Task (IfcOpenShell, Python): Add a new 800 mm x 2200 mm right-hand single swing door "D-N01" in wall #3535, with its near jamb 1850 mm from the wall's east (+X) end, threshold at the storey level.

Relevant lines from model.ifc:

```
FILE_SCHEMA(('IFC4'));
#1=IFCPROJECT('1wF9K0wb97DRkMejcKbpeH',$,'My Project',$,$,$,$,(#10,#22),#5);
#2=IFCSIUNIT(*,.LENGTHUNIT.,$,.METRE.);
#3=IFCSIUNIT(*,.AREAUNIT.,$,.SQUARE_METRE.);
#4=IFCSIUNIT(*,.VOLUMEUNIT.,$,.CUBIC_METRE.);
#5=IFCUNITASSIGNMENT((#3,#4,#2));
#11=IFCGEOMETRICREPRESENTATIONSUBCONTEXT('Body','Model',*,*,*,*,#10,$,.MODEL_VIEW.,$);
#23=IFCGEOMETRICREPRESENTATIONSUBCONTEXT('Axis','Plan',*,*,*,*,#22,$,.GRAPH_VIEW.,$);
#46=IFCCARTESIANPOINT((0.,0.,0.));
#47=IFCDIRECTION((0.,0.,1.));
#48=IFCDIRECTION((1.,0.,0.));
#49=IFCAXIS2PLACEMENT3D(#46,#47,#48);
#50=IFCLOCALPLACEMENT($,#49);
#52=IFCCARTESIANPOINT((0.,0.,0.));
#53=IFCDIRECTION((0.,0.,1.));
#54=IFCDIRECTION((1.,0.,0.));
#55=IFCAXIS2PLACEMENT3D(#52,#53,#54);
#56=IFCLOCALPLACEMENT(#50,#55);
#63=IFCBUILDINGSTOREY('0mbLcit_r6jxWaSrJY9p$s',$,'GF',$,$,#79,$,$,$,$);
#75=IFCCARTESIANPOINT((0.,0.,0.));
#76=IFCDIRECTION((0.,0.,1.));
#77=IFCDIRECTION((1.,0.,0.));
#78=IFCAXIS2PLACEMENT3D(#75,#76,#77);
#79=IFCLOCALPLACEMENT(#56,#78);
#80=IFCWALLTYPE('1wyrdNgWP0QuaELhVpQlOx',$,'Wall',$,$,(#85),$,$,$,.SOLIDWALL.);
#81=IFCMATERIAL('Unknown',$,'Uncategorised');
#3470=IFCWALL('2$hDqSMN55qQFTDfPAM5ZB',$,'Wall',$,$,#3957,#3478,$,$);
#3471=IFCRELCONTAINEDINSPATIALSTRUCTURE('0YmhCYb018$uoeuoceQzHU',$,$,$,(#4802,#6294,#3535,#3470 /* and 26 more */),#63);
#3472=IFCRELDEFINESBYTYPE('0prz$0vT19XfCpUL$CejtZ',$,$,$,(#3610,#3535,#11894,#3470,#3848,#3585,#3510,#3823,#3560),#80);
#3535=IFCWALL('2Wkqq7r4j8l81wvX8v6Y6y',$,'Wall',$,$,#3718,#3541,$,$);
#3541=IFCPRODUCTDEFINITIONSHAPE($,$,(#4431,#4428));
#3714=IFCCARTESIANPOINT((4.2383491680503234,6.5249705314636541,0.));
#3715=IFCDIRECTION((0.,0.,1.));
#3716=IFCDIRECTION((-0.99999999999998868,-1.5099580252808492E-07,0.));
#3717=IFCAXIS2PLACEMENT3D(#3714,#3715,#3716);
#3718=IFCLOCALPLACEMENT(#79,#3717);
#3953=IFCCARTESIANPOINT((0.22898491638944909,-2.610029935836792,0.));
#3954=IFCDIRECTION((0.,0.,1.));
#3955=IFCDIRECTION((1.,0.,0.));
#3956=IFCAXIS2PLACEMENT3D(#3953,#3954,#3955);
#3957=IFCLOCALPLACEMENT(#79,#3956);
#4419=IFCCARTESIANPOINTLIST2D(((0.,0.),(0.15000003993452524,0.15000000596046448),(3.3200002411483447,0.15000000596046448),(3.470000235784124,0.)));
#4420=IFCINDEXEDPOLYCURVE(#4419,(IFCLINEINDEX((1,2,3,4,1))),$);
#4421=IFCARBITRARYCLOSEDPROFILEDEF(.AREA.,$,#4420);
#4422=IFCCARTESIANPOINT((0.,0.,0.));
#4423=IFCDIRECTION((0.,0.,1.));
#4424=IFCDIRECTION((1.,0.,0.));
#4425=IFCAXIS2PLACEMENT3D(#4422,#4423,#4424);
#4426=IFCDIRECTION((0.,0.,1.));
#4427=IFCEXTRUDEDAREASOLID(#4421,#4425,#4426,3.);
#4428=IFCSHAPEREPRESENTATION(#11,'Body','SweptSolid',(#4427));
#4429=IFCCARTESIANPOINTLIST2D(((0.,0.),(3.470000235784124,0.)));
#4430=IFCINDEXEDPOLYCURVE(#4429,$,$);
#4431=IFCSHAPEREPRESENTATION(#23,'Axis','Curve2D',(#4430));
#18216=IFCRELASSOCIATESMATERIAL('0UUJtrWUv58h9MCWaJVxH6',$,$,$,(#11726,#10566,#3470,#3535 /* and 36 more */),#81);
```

```python
import numpy as np
import ifcopenshell
import ifcopenshell.api.feature
import ifcopenshell.api.geometry
import ifcopenshell.api.root
import ifcopenshell.api.spatial
import ifcopenshell.geom
import ifcopenshell.util.element
import ifcopenshell.util.placement
import ifcopenshell.util.representation
import ifcopenshell.util.shape
import ifcopenshell.util.unit

model = ifcopenshell.open("model.ifc")
unit_scale = ifcopenshell.util.unit.calculate_unit_scale(model)
settings = ifcopenshell.geom.settings()


def volume(element):
    """Net volume in cubic metres, openings subtracted."""
    shape = ifcopenshell.geom.create_shape(settings, element)
    return ifcopenshell.util.shape.get_volume(shape.geometry)


wall = model.by_guid("2Wkqq7r4j8l81wvX8v6Y6y")
storey = ifcopenshell.util.element.get_container(wall, ifc_class="IfcBuildingStorey")
context = ifcopenshell.util.representation.get_context(model, "Model", "Body", "MODEL_VIEW")
before = volume(wall)

width, height, from_end, sill = 0.8, 2.2, 1.85, 0.0  # metres

# The wall runs along its own X axis, and the end named is its -X end.
wall_shape = ifcopenshell.geom.create_shape(settings, wall)
x, y, z = ifcopenshell.util.shape.get_vertices(wall_shape.geometry).T
start = x.min() + from_end
face, thickness = float(y.min()), float(y.max() - y.min())
wall_matrix = ifcopenshell.util.placement.get_local_placement(wall.ObjectPlacement)
level = ifcopenshell.util.placement.get_local_placement(storey.ObjectPlacement)[2, 3]


def in_wall(x, y):
    """Placement at x, y metres in the wall's axes, at sill height."""
    matrix = wall_matrix.copy()
    matrix[:, 3] = wall_matrix @ np.array([x / unit_scale, y / unit_scale, 0.0, 1.0])
    matrix[2, 3] = level + sill / unit_scale
    return matrix


# Opening: a box that overshoots both wall faces by 50 mm.
opening = ifcopenshell.api.root.create_entity(model, ifc_class="IfcOpeningElement", predefined_type="OPENING")
box = ifcopenshell.api.geometry.add_wall_representation(
    model, context=context, length=width, height=height, thickness=thickness + 0.1
)
ifcopenshell.api.geometry.assign_representation(model, product=opening, representation=box)
ifcopenshell.api.geometry.edit_object_placement(model, product=opening, matrix=in_wall(start, face - 0.05), is_si=False)
ifcopenshell.api.feature.add_feature(model, feature=opening, element=wall)

door = ifcopenshell.api.root.create_entity(model, ifc_class="IfcDoor", name="D-N01", predefined_type="DOOR")
door.OverallWidth, door.OverallHeight = width / unit_scale, height / unit_scale
door.OperationType = "SINGLE_SWING_RIGHT"
body = ifcopenshell.api.geometry.add_door_representation(
    model,
    context=context,
    overall_width=door.OverallWidth,
    overall_height=door.OverallHeight,
    operation_type="SINGLE_SWING_RIGHT",
    lining_properties={"LiningDepth": thickness / unit_scale, "ThresholdDepth": thickness / unit_scale},
)
ifcopenshell.api.geometry.assign_representation(model, product=door, representation=body)
ifcopenshell.api.spatial.assign_container(model, products=[door], relating_structure=storey)
ifcopenshell.api.feature.add_filling(model, opening=opening, element=door)

# The lining spans the wall, so the door starts at the wall face.
ifcopenshell.api.geometry.edit_object_placement(model, product=door, matrix=in_wall(start, face), is_si=False)

after = volume(wall)

print(f"wall volume {before:.3f} -> {after:.3f} m3")

model.write("model_updated.ifc")
```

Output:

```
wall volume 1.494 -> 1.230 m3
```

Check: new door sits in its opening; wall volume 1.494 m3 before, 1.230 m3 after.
